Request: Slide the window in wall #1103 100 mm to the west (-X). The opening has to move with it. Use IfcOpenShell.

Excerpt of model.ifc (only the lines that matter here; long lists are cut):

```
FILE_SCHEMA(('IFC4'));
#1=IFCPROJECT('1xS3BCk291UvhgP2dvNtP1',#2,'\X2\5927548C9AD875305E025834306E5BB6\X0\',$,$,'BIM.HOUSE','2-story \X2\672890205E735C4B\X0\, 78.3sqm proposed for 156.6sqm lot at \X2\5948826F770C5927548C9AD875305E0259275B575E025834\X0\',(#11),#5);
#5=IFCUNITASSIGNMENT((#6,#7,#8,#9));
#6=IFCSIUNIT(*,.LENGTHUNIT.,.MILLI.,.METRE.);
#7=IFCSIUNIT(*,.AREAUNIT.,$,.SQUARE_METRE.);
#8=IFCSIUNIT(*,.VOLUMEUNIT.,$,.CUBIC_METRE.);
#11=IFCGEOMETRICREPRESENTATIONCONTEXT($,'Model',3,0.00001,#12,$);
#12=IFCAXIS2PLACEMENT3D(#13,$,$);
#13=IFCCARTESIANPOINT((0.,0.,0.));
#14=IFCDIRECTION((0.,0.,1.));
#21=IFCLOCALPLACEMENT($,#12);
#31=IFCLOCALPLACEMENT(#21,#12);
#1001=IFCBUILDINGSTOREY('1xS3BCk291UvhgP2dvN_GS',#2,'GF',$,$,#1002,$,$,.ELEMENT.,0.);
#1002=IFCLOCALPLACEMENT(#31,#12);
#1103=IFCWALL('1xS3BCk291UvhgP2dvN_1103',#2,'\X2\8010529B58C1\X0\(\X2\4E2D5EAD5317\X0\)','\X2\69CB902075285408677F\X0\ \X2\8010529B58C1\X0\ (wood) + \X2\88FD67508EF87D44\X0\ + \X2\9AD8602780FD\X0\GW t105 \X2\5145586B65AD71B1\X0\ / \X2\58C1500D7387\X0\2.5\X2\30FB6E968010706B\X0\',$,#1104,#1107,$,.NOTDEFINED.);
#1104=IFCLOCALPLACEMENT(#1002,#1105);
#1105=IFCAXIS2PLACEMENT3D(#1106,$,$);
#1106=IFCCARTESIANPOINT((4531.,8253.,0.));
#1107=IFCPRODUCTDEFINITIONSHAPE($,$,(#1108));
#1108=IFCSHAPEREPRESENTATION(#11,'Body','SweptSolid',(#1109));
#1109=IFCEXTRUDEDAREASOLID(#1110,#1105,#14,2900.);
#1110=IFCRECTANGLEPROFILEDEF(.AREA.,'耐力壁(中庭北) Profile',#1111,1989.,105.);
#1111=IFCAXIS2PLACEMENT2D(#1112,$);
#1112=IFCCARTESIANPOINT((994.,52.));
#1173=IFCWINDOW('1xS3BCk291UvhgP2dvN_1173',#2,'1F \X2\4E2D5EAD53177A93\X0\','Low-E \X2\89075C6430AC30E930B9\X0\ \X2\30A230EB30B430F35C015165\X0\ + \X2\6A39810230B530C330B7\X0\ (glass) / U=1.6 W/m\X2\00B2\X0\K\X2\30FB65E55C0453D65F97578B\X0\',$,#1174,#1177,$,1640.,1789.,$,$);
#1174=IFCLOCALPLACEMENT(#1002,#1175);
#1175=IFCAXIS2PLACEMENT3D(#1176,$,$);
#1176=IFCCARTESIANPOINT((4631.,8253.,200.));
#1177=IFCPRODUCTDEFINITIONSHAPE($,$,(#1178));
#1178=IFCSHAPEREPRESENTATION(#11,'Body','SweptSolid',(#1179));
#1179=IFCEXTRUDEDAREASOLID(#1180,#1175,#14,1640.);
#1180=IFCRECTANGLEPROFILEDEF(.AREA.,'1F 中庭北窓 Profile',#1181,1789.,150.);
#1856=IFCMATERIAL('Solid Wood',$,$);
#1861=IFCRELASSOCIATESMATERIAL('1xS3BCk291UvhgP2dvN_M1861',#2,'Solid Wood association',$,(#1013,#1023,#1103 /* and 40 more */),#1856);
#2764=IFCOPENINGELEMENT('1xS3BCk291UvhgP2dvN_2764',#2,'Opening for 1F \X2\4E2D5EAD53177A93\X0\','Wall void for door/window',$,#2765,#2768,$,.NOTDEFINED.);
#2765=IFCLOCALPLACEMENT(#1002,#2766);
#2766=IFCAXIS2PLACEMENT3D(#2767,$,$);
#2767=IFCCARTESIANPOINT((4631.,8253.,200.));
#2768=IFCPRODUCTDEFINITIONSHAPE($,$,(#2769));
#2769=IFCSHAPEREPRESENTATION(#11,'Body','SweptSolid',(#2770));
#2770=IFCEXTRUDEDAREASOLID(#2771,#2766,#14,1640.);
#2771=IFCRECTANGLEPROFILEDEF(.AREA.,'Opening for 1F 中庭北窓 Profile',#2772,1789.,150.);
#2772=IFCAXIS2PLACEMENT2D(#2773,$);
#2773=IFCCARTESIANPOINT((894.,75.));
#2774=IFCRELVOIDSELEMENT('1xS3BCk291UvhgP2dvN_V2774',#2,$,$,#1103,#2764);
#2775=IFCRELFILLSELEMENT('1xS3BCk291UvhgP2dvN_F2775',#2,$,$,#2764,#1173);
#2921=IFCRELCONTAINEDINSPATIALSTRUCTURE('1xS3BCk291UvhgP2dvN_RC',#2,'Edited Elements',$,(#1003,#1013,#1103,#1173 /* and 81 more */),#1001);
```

```python
import ifcopenshell
import ifcopenshell.api.geometry
import ifcopenshell.util.placement
import ifcopenshell.util.unit

model = ifcopenshell.open("model.ifc")
unit_scale = ifcopenshell.util.unit.calculate_unit_scale(model)

window = model.by_id(1173)
opening = window.FillsVoids[0].RelatingOpeningElement
wall = opening.VoidsElements[0].RelatingBuildingElement

wall_matrix = ifcopenshell.util.placement.get_local_placement(wall.ObjectPlacement)
shift = wall_matrix[:3, 0] * -0.1 / unit_scale
before = ifcopenshell.util.placement.get_local_placement(window.ObjectPlacement)[:3, 3].copy()

# The window is not placed relative to its opening, so move both.
for product in (opening, window):
    matrix = ifcopenshell.util.placement.get_local_placement(product.ObjectPlacement)
    matrix[:3, 3] += shift
    ifcopenshell.api.geometry.edit_object_placement(model, product=product, matrix=matrix, is_si=False)

after = ifcopenshell.util.placement.get_local_placement(window.ObjectPlacement)[:3, 3]
print("window moved by", (after - before).round(3) + 0.0)

model.write("model_edited.ifc")
```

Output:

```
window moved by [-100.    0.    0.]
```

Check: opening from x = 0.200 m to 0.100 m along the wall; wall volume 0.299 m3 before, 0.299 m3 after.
